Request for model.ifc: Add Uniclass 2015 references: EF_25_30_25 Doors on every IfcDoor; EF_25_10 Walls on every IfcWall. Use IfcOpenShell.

First a look at what the model holds.

```python
import ifcopenshell

model = ifcopenshell.open("model.ifc")
print(model.schema)
print("classifications:", [c.Name for c in model.by_type("IfcClassification")])
for ifc_class in ("IfcDoor", "IfcRoof", "IfcStair", "IfcWall", "IfcWindow"):
    print(ifc_class, len(model.by_type(ifc_class)))
```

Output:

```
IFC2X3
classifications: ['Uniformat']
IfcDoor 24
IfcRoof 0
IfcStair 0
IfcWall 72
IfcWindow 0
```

```python
import ifcopenshell
import ifcopenshell.api.classification

model = ifcopenshell.open("model.ifc")

# IFC2X3 requires Source and Edition and has no link from the project to the system.
system = model.create_entity("IfcClassification", Source="NBS", Edition="2015", Name="Uniclass 2015")

codes = {
    "IfcDoor": ("EF_25_30_25", "Doors"),
    "IfcWall": ("EF_25_10", "Walls"),
}
for ifc_class, (code, name) in codes.items():
    products = model.by_type(ifc_class)
    ifcopenshell.api.classification.add_reference(
        model, products=products, classification=system, identification=code, name=name
    )
    print(code, len(products))

model.write("model_edited.ifc")
```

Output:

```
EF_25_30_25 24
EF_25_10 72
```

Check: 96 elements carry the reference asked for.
